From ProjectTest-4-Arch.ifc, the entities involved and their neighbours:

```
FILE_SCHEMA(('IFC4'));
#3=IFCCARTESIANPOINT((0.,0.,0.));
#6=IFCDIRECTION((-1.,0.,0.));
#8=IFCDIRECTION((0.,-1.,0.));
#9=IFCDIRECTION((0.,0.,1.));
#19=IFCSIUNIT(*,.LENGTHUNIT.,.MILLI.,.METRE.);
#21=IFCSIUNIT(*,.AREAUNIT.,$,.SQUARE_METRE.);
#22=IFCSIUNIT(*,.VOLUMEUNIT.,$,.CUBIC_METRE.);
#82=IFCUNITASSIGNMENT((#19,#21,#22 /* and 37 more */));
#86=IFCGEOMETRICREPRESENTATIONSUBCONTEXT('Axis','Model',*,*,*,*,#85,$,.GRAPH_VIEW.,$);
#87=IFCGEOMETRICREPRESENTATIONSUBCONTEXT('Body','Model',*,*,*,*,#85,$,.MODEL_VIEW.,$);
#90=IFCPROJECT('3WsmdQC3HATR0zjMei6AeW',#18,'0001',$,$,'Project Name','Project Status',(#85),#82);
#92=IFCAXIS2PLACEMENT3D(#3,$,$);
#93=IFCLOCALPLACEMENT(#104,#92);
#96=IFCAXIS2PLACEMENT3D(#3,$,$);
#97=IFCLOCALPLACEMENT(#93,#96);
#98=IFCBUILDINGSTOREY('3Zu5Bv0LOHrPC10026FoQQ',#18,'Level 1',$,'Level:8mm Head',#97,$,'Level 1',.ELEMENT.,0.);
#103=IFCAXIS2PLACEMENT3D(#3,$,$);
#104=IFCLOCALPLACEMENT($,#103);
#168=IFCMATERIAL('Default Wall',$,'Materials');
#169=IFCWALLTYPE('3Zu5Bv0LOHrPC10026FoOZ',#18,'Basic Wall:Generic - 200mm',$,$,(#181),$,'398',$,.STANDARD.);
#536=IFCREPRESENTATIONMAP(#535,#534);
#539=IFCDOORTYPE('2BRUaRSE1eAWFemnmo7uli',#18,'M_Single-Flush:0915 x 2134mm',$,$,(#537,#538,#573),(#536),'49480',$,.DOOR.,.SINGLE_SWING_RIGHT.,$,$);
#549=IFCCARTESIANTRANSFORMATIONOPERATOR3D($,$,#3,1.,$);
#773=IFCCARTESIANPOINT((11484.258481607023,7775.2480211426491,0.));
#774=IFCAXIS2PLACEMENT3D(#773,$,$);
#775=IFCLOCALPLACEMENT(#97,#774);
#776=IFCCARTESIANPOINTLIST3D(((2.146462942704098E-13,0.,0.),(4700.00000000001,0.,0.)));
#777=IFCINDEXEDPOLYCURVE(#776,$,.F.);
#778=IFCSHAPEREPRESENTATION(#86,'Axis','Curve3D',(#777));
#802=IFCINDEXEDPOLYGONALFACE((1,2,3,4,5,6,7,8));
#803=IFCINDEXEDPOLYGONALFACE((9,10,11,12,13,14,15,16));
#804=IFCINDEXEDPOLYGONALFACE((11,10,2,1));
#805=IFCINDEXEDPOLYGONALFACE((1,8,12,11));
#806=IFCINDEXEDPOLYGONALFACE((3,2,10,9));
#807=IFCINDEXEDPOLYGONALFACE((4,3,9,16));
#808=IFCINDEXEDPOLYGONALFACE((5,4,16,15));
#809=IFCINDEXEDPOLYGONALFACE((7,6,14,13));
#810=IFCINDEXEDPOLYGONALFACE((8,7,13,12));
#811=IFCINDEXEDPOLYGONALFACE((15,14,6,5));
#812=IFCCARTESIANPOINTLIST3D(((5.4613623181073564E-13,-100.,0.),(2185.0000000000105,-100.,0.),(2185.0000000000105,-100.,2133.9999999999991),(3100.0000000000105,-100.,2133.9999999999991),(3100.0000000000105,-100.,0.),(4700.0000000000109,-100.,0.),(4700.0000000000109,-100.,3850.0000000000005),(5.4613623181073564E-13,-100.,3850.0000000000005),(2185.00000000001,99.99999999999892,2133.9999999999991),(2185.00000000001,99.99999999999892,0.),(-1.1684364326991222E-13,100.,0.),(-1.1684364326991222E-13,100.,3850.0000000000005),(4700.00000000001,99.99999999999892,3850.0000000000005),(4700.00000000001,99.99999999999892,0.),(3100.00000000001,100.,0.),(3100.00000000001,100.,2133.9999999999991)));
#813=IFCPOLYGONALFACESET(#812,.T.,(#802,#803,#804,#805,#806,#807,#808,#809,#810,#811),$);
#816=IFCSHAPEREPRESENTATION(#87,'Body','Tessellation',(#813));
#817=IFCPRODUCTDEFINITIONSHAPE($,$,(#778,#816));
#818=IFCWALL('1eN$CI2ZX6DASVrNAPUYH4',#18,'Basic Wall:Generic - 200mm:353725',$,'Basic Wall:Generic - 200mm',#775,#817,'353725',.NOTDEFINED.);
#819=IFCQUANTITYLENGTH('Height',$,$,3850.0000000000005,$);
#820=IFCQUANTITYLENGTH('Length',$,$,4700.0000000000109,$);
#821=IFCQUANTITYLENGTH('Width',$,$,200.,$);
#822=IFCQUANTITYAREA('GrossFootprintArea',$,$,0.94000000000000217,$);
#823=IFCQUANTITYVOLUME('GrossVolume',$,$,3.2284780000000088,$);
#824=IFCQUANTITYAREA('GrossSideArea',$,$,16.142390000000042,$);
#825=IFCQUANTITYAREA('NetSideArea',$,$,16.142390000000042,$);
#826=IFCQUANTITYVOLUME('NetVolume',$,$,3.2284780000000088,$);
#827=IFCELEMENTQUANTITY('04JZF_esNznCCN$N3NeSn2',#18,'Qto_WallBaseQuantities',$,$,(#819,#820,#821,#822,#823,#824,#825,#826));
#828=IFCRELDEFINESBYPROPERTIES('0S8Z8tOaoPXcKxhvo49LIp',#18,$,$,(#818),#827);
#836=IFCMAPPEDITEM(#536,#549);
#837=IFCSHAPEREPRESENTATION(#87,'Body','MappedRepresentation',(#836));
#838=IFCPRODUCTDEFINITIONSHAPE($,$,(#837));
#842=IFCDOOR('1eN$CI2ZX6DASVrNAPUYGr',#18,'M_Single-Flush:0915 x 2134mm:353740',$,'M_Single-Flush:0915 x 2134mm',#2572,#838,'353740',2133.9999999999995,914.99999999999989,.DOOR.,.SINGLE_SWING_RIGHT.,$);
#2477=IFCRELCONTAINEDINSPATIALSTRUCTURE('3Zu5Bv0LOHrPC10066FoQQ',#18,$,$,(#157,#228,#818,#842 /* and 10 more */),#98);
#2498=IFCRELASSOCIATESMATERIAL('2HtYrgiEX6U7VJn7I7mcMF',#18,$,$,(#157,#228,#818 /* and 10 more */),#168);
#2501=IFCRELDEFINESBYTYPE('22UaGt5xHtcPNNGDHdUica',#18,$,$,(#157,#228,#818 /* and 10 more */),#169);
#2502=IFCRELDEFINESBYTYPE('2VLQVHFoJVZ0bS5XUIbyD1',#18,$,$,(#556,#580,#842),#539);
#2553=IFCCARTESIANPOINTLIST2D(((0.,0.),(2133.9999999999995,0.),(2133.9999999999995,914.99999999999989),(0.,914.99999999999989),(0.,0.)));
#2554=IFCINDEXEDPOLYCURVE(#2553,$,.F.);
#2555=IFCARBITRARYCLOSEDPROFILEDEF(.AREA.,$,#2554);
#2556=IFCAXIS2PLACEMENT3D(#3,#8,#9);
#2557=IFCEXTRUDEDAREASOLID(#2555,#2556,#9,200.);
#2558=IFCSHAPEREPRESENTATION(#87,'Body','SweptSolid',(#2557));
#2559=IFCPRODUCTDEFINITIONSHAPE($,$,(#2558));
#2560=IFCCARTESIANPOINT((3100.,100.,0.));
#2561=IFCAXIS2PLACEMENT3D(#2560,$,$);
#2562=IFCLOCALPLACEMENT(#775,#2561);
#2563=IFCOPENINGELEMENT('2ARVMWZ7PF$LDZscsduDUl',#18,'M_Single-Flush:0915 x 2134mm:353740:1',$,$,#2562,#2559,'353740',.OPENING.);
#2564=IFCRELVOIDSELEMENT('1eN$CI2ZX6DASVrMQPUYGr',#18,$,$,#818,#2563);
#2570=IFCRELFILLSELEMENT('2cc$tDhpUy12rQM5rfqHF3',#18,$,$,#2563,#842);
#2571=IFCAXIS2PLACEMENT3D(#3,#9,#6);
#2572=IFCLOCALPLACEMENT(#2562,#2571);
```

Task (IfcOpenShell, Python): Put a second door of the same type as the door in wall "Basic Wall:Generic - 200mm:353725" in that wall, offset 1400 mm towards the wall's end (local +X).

```python
import ifcopenshell
import ifcopenshell.api.feature
import ifcopenshell.api.geometry
import ifcopenshell.api.pset
import ifcopenshell.api.root
import ifcopenshell.geom
import ifcopenshell.util.element
import ifcopenshell.util.placement
import ifcopenshell.util.shape
import ifcopenshell.util.unit

model = ifcopenshell.open("ProjectTest-4-Arch.ifc")
unit_scale = ifcopenshell.util.unit.calculate_unit_scale(model)
area_scale = ifcopenshell.util.unit.calculate_unit_scale(model, "AREAUNIT")
volume_scale = ifcopenshell.util.unit.calculate_unit_scale(model, "VOLUMEUNIT")
settings = ifcopenshell.geom.settings()


def volume(element):
    """Net volume in cubic metres, openings subtracted."""
    shape = ifcopenshell.geom.create_shape(settings, element)
    return ifcopenshell.util.shape.get_volume(shape.geometry)


def reuse_history(source, copy):
    """copy_class also copies each property set's owner history, people and application; keep the originals."""
    for rel in copy.IsDefinedBy:
        if rel.is_a("IfcRelDefinesByProperties") and (history := rel.RelatingPropertyDefinition.OwnerHistory):
            rel.RelatingPropertyDefinition.OwnerHistory = source.OwnerHistory
            ifcopenshell.util.element.remove_deep2(model, history)


door = model.by_guid("1eN$CI2ZX6DASVrNAPUYGr")
opening = door.FillsVoids[0].RelatingOpeningElement
wall = opening.VoidsElements[0].RelatingBuildingElement
before = volume(wall)
shift = ifcopenshell.util.placement.get_local_placement(wall.ObjectPlacement)[:3, 0] * 1.4 / unit_scale

# copy_class copies the void relationship, type, container and properties, but no geometry.
new_opening = ifcopenshell.api.root.copy_class(model, product=opening)
new_opening.Representation = ifcopenshell.util.element.copy_deep(
    model, opening.Representation, exclude=["IfcGeometricRepresentationContext", "IfcRepresentationMap"]
)
new_opening.Name = "M_Single-Flush:0915 x 2134mm"
new_opening.Tag = None
reuse_history(opening, new_opening)
new_door = ifcopenshell.api.root.copy_class(model, product=door)
new_door.Representation = ifcopenshell.util.element.copy_deep(
    model, door.Representation, exclude=["IfcGeometricRepresentationContext", "IfcRepresentationMap"]
)
new_door.Name = "M_Single-Flush:0915 x 2134mm"
new_door.Tag = None
reuse_history(door, new_door)
ifcopenshell.api.feature.add_filling(model, opening=new_opening, element=new_door)

for old, new in ((opening, new_opening), (door, new_door)):
    matrix = ifcopenshell.util.placement.get_local_placement(old.ObjectPlacement)
    matrix[:3, 3] += shift
    ifcopenshell.api.geometry.edit_object_placement(model, product=new, matrix=matrix, is_si=False)

after = volume(wall)
thickness = 0.2  # wall thickness in metres

# Update the wall's stored quantities.
qto = model.by_id(ifcopenshell.util.element.get_pset(wall, "Qto_WallBaseQuantities", should_inherit=False)["id"])
ifcopenshell.api.pset.edit_qto(model, qto=qto, properties={
    "NetSideArea": after / thickness / area_scale,
    "NetVolume": after / volume_scale,
})

print(f"wall volume {before:.3f} -> {after:.3f} m3")

model.write("ProjectTest-4-Arch-out.ifc")
```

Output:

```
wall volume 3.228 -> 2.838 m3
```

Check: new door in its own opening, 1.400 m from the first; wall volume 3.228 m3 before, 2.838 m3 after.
